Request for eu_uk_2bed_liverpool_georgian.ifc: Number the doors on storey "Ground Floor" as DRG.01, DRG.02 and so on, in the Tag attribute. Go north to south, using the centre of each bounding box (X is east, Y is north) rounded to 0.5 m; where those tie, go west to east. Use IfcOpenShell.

First a look at what the model holds.

```python
import ifcopenshell
import ifcopenshell.util.element
import ifcopenshell.util.placement

model = ifcopenshell.open("eu_uk_2bed_liverpool_georgian.ifc")
print(model.schema)
storey = next(s for s in model.by_type("IfcBuildingStorey") if s.Name == "Ground Floor")
doors = [e for e in ifcopenshell.util.element.get_decomposition(storey) if e.is_a("IfcDoor")]
for e in sorted(doors, key=lambda e: e.id()):
    origin = ifcopenshell.util.placement.get_local_placement(e.ObjectPlacement)[:3, 3]
    print(e.id(), e.Tag, e.Name, origin.round(2) + 0.0, sep=" | ")
```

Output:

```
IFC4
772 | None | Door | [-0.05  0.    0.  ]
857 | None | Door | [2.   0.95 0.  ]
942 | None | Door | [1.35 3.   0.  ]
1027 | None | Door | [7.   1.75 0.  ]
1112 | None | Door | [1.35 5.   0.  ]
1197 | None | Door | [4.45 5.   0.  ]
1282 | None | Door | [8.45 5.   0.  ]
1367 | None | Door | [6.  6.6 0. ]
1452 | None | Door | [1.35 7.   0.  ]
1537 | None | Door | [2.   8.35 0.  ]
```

```python
import ifcopenshell
import ifcopenshell.geom
import ifcopenshell.util.element
import ifcopenshell.util.shape

model = ifcopenshell.open("eu_uk_2bed_liverpool_georgian.ifc")
settings = ifcopenshell.geom.settings()
settings.set("use-world-coords", True)


def centre(element):
    shape = ifcopenshell.geom.create_shape(settings, element)
    return ifcopenshell.util.shape.get_bbox_centroid(shape.geometry)


storey = next(s for s in model.by_type("IfcBuildingStorey") if s.Name == "Ground Floor")
doors = [e for e in ifcopenshell.util.element.get_decomposition(storey) if e.is_a("IfcDoor")]

# Insertion points can sit at a corner or the storey origin, so sort by the geometry (in metres).
centres = {e: centre(e) for e in doors}
doors.sort(key=lambda e: (-round(centres[e][1] / 0.5), centres[e][0]))

for i, e in enumerate(doors, start=1):
    number = f"DRG.{i:02d}"
    e.Tag = number
    print(e.id(), number)

model.write("eu_uk_2bed_liverpool_georgian_updated.ifc")
```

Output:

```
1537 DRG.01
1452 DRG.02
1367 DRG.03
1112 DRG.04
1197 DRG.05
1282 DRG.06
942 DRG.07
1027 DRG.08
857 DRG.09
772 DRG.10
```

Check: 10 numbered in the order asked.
